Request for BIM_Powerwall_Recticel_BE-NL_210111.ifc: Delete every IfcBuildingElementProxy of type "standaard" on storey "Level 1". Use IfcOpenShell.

First a look at what the model holds.

```python
import ifcopenshell
import ifcopenshell.util.element

model = ifcopenshell.open("BIM_Powerwall_Recticel_BE-NL_210111.ifc")
print(model.schema)
storey = next(s for s in model.by_type("IfcBuildingStorey") if s.Name == "Level 1")
proxies = [e for e in ifcopenshell.util.element.get_decomposition(storey) if e.is_a("IfcBuildingElementProxy")]
seen = {}
for e in proxies:
    element_type = ifcopenshell.util.element.get_type(e)
    name = element_type.Name if element_type not in (None, e) else None
    seen[name] = seen.get(name, 0) + 1
for name, count in sorted(seen.items(), key=str):
    print(count, "x", name)
```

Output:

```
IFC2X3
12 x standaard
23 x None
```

```python
import ifcopenshell
import ifcopenshell.api.root
import ifcopenshell.util.element

model = ifcopenshell.open("BIM_Powerwall_Recticel_BE-NL_210111.ifc")

storey = next(s for s in model.by_type("IfcBuildingStorey") if s.Name == "Level 1")
proxies = [e for e in ifcopenshell.util.element.get_decomposition(storey) if e.is_a("IfcBuildingElementProxy")]
targets = [e for e in proxies if (t := ifcopenshell.util.element.get_type(e)) not in (None, e) and t.Name == "standaard"]

for e in targets:
    ifcopenshell.api.root.remove_product(model, product=e)
print(len(targets), "removed")

model.write("BIM_Powerwall_Recticel_BE-NL_210111_edited.ifc")
```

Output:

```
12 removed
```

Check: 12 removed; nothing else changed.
